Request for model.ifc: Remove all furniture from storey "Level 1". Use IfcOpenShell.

First a look at what the model holds.

```python
import ifcopenshell
import ifcopenshell.util.element

model = ifcopenshell.open("model.ifc")
print(model.schema)
storey = next(s for s in model.by_type("IfcBuildingStorey") if s.Name == "Level 1")
furniture = [e for e in ifcopenshell.util.element.get_decomposition(storey) if e.is_a("IfcFurnishingElement")]
seen = {}
for e in furniture:
    element_type = ifcopenshell.util.element.get_type(e)
    name = element_type.Name if element_type not in (None, e) else None
    seen[name] = seen.get(name, 0) + 1
for name, count in sorted(seen.items(), key=str):
    print(count, "x", name)
```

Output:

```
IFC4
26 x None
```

```python
import ifcopenshell
import ifcopenshell.api.root
import ifcopenshell.util.element

model = ifcopenshell.open("model.ifc")

storey = next(s for s in model.by_type("IfcBuildingStorey") if s.Name == "Level 1")
furniture = [e for e in ifcopenshell.util.element.get_decomposition(storey) if e.is_a("IfcFurnishingElement")]

for e in furniture:
    ifcopenshell.api.root.remove_product(model, product=e)
print(len(furniture), "removed")

model.write("model_updated.ifc")
```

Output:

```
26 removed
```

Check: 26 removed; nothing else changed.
